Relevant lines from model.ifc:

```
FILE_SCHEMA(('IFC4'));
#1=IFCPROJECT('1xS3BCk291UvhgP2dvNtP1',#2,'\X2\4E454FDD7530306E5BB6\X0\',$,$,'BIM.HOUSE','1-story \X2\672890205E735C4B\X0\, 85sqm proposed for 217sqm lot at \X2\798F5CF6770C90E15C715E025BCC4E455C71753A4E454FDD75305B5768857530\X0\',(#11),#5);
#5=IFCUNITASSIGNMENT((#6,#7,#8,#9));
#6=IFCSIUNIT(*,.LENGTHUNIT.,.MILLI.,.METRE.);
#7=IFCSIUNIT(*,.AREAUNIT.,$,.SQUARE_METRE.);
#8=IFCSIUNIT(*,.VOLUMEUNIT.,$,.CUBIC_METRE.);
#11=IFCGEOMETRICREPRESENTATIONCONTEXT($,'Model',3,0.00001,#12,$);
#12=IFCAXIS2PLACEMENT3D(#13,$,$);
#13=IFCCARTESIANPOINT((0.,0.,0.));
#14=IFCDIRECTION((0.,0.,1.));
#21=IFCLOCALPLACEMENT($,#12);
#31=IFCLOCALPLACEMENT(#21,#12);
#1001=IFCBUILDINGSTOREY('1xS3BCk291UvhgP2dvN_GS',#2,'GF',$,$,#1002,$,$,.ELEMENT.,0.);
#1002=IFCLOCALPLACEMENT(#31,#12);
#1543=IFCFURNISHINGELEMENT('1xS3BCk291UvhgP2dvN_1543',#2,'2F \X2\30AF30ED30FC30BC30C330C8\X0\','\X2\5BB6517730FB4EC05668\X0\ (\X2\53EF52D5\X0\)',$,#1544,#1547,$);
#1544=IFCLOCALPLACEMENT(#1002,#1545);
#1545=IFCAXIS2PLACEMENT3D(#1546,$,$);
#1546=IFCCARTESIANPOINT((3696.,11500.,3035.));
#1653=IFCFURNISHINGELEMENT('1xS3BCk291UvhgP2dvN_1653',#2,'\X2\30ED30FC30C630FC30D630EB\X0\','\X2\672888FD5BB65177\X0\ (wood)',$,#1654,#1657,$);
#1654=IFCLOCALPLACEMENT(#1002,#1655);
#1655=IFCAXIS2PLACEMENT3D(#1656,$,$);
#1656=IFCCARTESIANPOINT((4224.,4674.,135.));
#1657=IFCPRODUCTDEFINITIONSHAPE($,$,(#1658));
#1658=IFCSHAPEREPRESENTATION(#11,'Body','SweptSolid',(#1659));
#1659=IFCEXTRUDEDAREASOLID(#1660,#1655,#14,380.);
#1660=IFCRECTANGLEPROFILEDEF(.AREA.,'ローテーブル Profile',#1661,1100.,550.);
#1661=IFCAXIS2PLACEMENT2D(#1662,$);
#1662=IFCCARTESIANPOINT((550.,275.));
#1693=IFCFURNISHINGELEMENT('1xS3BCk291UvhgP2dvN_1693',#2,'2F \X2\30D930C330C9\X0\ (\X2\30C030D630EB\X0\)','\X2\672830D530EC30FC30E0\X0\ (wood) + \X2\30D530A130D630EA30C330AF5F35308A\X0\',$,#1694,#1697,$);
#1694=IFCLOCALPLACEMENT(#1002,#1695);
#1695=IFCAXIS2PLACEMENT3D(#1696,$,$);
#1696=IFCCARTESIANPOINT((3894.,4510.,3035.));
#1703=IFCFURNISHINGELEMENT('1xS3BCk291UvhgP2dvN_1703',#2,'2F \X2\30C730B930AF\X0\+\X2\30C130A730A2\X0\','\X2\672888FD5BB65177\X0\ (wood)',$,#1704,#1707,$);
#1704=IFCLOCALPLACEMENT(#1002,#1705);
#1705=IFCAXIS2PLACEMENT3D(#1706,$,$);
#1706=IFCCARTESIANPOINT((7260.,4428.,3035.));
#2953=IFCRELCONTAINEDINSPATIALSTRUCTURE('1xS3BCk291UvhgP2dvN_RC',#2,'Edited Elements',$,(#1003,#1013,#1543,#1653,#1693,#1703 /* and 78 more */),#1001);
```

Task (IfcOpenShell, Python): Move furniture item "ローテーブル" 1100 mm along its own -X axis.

```python
import ifcopenshell
import ifcopenshell.api.geometry
import ifcopenshell.util.placement

model = ifcopenshell.open("model.ifc")

item = model.by_guid("1xS3BCk291UvhgP2dvN_1653")
matrix = ifcopenshell.util.placement.get_local_placement(item.ObjectPlacement)
matrix[:3, 3] -= matrix[:3, 0] * 1100.0
ifcopenshell.api.geometry.edit_object_placement(model, product=item, matrix=matrix, is_si=False)

print(ifcopenshell.util.placement.get_local_placement(item.ObjectPlacement).round(3) + 0.0)

model.write("model_edited.ifc")
```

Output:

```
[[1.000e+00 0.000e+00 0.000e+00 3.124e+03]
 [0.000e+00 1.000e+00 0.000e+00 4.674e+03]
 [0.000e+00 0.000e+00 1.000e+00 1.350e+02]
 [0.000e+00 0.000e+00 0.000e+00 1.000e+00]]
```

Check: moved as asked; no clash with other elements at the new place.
